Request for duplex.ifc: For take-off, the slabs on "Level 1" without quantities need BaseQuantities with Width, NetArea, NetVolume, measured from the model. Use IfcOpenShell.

First a look at what the model holds.

```python
import ifcopenshell
import ifcopenshell.util.element
import ifcopenshell.util.unit

model = ifcopenshell.open("duplex.ifc")
print(model.schema)
for unit_type in ("LENGTHUNIT", "AREAUNIT", "VOLUMEUNIT"):
    print(unit_type, ifcopenshell.util.unit.calculate_unit_scale(model, unit_type))
storey = next(s for s in model.by_type("IfcBuildingStorey") if s.Name == "Level 1")
slabs = [e for e in ifcopenshell.util.element.get_decomposition(storey) if e.is_a("IfcSlab")]
for e in sorted(slabs, key=lambda e: e.id()):
    print(e.id(), e.is_a(), e.Name, list(ifcopenshell.util.element.get_psets(e, qtos_only=True)), sep=" | ")
```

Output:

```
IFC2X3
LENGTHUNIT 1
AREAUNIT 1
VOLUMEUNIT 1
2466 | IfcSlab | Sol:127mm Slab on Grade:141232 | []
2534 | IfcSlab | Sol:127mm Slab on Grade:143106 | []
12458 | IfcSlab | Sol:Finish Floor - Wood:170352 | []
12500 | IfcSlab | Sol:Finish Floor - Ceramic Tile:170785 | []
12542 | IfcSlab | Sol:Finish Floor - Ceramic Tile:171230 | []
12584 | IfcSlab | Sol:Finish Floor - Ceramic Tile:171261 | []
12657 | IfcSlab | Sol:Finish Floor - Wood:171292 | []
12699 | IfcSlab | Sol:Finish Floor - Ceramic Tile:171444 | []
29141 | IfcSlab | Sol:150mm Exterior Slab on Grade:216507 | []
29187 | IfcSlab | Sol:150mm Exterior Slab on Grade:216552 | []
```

```python
import ifcopenshell
import ifcopenshell.api.pset
import ifcopenshell.geom
import ifcopenshell.util.element
import ifcopenshell.util.shape
import ifcopenshell.util.unit

model = ifcopenshell.open("duplex.ifc")
unit_scale = ifcopenshell.util.unit.calculate_unit_scale(model)
area_scale = ifcopenshell.util.unit.calculate_unit_scale(model, "AREAUNIT")
volume_scale = ifcopenshell.util.unit.calculate_unit_scale(model, "VOLUMEUNIT")
settings = ifcopenshell.geom.settings()

storey = next(s for s in model.by_type("IfcBuildingStorey") if s.Name == "Level 1")
slabs = [e for e in ifcopenshell.util.element.get_decomposition(storey) if e.is_a("IfcSlab")]

for e in sorted(slabs, key=lambda e: e.id()):
    if ifcopenshell.util.element.get_psets(e, qtos_only=True, should_inherit=False):
        continue
    # Geometry comes back in metres, in the element's own axes.
    shape = ifcopenshell.geom.create_shape(settings, e)
    values = {
        "Width": ifcopenshell.util.shape.get_z(shape.geometry) / unit_scale,
        "NetArea": ifcopenshell.util.shape.get_footprint_area(shape.geometry) / area_scale,
        "NetVolume": ifcopenshell.util.shape.get_volume(shape.geometry) / volume_scale,
    }
    qto = ifcopenshell.api.pset.add_qto(model, product=e, name="BaseQuantities")
    ifcopenshell.api.pset.edit_qto(model, qto=qto, properties=values)
    print(e.id(), {k: round(v, 3) for k, v in values.items()})

model.write("duplex_edited.ifc")
```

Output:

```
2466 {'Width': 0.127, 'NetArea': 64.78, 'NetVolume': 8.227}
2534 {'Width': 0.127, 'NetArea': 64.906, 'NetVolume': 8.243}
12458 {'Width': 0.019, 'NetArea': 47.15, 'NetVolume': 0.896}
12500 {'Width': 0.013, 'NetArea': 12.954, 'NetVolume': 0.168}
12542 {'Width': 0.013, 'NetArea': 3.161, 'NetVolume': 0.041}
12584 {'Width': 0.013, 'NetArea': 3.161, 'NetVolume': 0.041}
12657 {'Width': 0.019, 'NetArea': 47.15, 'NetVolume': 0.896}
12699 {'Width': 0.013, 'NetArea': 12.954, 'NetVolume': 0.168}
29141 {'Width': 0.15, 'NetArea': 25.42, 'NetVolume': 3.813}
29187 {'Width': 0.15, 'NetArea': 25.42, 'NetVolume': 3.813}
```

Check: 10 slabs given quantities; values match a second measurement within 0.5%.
